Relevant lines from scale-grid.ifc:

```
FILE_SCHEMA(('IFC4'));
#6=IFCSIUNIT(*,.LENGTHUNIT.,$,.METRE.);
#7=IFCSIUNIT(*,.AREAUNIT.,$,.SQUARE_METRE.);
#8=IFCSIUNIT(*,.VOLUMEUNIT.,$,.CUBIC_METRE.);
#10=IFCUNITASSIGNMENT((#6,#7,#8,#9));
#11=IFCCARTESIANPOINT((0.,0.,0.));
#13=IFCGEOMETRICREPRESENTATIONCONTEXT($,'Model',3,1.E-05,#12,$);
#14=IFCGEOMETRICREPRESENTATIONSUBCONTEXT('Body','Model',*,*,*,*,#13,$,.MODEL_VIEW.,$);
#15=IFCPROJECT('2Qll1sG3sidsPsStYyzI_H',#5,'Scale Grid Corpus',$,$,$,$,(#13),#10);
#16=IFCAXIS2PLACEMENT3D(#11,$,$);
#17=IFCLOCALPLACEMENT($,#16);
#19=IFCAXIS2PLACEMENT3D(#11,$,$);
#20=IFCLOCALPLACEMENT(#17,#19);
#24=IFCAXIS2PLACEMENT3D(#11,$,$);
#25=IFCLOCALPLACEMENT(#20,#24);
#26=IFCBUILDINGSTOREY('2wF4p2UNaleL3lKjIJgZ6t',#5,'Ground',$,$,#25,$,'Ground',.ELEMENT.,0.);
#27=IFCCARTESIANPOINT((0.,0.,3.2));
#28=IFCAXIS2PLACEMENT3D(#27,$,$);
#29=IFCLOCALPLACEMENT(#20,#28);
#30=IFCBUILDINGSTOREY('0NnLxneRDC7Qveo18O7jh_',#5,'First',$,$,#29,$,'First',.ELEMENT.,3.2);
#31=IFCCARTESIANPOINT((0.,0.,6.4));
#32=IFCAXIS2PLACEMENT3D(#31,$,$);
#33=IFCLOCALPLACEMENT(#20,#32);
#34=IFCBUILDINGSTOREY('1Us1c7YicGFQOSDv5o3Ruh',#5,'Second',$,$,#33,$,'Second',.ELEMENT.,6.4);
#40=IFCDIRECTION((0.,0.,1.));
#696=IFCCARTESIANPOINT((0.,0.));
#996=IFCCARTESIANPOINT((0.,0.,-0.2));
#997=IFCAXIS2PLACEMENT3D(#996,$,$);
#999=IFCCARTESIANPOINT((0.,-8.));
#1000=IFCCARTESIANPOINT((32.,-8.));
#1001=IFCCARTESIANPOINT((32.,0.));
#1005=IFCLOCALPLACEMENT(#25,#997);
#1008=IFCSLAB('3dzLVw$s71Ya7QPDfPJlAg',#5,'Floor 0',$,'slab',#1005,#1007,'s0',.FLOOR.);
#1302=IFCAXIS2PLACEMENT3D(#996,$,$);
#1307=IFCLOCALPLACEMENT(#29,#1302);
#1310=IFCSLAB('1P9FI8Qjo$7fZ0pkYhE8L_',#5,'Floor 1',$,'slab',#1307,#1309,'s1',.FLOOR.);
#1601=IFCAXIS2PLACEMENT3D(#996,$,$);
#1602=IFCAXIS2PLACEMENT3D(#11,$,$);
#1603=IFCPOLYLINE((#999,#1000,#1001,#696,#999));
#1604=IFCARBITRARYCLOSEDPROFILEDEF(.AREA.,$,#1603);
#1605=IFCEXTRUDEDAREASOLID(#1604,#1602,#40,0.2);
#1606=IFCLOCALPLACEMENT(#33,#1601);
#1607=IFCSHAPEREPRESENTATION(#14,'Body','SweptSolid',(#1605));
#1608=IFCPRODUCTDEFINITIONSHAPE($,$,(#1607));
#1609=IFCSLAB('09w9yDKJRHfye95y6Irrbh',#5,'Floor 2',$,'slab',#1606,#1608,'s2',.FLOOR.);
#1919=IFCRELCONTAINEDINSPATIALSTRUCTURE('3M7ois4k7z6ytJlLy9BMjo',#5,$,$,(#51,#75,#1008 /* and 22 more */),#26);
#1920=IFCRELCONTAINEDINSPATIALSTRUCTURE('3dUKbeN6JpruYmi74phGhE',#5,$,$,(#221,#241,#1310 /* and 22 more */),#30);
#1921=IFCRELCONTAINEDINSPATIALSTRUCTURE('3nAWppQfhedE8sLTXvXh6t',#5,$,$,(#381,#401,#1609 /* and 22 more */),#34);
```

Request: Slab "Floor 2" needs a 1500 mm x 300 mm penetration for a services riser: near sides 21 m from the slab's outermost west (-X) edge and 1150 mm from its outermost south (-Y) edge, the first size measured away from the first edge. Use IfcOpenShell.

```python
import numpy as np
import ifcopenshell
import ifcopenshell.api.feature
import ifcopenshell.api.geometry
import ifcopenshell.api.root
import ifcopenshell.geom
import ifcopenshell.util.placement
import ifcopenshell.util.representation
import ifcopenshell.util.shape
import ifcopenshell.util.unit

model = ifcopenshell.open("scale-grid.ifc")
unit_scale = ifcopenshell.util.unit.calculate_unit_scale(model)
settings = ifcopenshell.geom.settings()


def volume(element):
    """Net volume in cubic metres, openings subtracted."""
    shape = ifcopenshell.geom.create_shape(settings, element)
    return ifcopenshell.util.shape.get_volume(shape.geometry)


slab = model.by_guid("09w9yDKJRHfye95y6Irrbh")
before = volume(slab)

# Extent in the slab's own axes, in metres. The edges named are its -X and -Y sides.
slab_shape = ifcopenshell.geom.create_shape(settings, slab)
vertices = ifcopenshell.util.shape.get_vertices(slab_shape.geometry)
x_min, y_min, bottom = vertices.min(axis=0)
top = vertices[:, 2].max()

opening = ifcopenshell.api.root.create_entity(model, ifc_class="IfcOpeningElement", name="Services riser opening", predefined_type="OPENING")
context = ifcopenshell.util.representation.get_context(model, "Model", "Body", "MODEL_VIEW")
width, depth = 1.5, 0.3
outline = [(0.0, 0.0), (width, 0.0), (width, depth), (0.0, depth), (0.0, 0.0)]
# Overshoot both faces by 50 mm so the cut is clean.
shape = ifcopenshell.api.geometry.add_slab_representation(
    model, context=context, depth=top - bottom + 0.1, polyline=outline
)
ifcopenshell.api.geometry.assign_representation(model, product=opening, representation=shape)

matrix = ifcopenshell.util.placement.get_local_placement(slab.ObjectPlacement)
matrix[:, 3] = matrix @ np.append(np.array([x_min + 21, y_min + 1.15, bottom - 0.05]) / unit_scale, 1.0)
ifcopenshell.api.geometry.edit_object_placement(model, product=opening, matrix=matrix, is_si=False)
ifcopenshell.api.feature.add_feature(model, feature=opening, element=slab)

after = volume(slab)

print(f"slab volume {before:.3f} -> {after:.3f} m3")

model.write("scale-grid-out.ifc")
```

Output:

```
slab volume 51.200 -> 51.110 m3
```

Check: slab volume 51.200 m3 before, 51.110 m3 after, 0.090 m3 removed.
